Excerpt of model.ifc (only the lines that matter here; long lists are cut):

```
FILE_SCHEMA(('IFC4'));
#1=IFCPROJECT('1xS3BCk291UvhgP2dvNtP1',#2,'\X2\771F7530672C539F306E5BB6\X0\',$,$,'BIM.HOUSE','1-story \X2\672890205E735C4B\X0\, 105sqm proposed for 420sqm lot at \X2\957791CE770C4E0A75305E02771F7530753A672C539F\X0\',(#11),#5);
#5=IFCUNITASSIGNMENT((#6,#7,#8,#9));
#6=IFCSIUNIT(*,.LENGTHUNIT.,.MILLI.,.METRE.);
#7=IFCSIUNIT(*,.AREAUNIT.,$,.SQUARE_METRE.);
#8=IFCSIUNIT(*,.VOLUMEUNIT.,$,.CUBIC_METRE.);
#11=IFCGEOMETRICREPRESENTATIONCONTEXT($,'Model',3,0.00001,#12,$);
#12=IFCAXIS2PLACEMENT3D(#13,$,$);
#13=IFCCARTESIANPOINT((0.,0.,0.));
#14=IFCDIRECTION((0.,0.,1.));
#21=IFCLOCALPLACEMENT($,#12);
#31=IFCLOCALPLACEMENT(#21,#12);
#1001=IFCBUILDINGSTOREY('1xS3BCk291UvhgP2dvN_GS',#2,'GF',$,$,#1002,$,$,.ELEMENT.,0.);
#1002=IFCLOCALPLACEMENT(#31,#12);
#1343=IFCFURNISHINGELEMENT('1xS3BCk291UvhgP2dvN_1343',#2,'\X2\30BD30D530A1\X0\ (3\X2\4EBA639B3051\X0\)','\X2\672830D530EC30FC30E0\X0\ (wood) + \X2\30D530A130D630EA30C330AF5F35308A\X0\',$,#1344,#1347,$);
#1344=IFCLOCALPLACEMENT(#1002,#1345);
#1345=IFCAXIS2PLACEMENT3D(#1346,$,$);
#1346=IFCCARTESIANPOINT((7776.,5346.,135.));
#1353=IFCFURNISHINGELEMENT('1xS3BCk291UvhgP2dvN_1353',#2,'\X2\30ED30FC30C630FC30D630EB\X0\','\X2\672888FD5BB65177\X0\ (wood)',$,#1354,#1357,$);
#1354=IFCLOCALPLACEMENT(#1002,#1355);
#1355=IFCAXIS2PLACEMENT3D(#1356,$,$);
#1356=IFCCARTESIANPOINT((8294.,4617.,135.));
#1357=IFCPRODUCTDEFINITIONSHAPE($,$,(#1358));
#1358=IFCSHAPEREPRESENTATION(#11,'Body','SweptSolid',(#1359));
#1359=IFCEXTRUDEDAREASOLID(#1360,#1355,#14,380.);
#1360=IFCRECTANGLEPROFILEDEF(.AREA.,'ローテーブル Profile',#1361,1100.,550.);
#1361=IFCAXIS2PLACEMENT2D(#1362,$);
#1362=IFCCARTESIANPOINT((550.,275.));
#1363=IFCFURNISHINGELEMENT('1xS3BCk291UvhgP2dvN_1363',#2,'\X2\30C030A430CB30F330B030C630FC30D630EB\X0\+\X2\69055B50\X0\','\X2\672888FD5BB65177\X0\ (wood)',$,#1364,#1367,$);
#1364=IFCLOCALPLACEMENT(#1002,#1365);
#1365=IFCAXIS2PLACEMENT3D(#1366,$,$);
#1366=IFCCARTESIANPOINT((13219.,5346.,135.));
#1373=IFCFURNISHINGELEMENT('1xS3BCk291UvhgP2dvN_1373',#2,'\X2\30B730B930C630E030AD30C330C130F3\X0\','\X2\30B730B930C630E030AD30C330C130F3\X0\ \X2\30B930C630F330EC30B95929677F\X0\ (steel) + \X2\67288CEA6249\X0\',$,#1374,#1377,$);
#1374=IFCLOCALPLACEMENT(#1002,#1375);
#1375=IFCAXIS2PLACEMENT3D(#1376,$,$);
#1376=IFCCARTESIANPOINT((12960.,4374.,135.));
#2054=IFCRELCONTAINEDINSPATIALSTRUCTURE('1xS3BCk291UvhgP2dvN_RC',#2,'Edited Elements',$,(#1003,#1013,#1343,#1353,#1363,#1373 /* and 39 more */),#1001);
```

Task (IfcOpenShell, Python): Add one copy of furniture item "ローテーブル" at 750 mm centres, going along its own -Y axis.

```python
import ifcopenshell
import ifcopenshell.api.geometry
import ifcopenshell.api.root
import ifcopenshell.util.element
import ifcopenshell.util.placement

model = ifcopenshell.open("model.ifc")


def reuse_history(source, copy):
    """copy_class also copies each property set's owner history, people and application; keep the originals."""
    for rel in copy.IsDefinedBy:
        if rel.is_a("IfcRelDefinesByProperties") and (history := rel.RelatingPropertyDefinition.OwnerHistory):
            rel.RelatingPropertyDefinition.OwnerHistory = source.OwnerHistory
            ifcopenshell.util.element.remove_deep2(model, history)


source = model.by_id(1353)
base = ifcopenshell.util.placement.get_local_placement(source.ObjectPlacement)
step = -base[:3, 1] * 750.0

for i in range(1, 2):
    copy = ifcopenshell.api.root.copy_class(model, product=source)
    copy.Representation = ifcopenshell.util.element.copy_deep(
        model, source.Representation, exclude=["IfcGeometricRepresentationContext", "IfcRepresentationMap"]
    )
    reuse_history(source, copy)
    matrix = base.copy()
    matrix[:3, 3] += i * step
    print("added at", matrix[:3, 3].round(3) + 0.0)
    ifcopenshell.api.geometry.edit_object_placement(model, product=copy, matrix=matrix, is_si=False)

model.write("model_v2.ifc")
```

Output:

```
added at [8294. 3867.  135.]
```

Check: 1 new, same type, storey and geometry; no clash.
